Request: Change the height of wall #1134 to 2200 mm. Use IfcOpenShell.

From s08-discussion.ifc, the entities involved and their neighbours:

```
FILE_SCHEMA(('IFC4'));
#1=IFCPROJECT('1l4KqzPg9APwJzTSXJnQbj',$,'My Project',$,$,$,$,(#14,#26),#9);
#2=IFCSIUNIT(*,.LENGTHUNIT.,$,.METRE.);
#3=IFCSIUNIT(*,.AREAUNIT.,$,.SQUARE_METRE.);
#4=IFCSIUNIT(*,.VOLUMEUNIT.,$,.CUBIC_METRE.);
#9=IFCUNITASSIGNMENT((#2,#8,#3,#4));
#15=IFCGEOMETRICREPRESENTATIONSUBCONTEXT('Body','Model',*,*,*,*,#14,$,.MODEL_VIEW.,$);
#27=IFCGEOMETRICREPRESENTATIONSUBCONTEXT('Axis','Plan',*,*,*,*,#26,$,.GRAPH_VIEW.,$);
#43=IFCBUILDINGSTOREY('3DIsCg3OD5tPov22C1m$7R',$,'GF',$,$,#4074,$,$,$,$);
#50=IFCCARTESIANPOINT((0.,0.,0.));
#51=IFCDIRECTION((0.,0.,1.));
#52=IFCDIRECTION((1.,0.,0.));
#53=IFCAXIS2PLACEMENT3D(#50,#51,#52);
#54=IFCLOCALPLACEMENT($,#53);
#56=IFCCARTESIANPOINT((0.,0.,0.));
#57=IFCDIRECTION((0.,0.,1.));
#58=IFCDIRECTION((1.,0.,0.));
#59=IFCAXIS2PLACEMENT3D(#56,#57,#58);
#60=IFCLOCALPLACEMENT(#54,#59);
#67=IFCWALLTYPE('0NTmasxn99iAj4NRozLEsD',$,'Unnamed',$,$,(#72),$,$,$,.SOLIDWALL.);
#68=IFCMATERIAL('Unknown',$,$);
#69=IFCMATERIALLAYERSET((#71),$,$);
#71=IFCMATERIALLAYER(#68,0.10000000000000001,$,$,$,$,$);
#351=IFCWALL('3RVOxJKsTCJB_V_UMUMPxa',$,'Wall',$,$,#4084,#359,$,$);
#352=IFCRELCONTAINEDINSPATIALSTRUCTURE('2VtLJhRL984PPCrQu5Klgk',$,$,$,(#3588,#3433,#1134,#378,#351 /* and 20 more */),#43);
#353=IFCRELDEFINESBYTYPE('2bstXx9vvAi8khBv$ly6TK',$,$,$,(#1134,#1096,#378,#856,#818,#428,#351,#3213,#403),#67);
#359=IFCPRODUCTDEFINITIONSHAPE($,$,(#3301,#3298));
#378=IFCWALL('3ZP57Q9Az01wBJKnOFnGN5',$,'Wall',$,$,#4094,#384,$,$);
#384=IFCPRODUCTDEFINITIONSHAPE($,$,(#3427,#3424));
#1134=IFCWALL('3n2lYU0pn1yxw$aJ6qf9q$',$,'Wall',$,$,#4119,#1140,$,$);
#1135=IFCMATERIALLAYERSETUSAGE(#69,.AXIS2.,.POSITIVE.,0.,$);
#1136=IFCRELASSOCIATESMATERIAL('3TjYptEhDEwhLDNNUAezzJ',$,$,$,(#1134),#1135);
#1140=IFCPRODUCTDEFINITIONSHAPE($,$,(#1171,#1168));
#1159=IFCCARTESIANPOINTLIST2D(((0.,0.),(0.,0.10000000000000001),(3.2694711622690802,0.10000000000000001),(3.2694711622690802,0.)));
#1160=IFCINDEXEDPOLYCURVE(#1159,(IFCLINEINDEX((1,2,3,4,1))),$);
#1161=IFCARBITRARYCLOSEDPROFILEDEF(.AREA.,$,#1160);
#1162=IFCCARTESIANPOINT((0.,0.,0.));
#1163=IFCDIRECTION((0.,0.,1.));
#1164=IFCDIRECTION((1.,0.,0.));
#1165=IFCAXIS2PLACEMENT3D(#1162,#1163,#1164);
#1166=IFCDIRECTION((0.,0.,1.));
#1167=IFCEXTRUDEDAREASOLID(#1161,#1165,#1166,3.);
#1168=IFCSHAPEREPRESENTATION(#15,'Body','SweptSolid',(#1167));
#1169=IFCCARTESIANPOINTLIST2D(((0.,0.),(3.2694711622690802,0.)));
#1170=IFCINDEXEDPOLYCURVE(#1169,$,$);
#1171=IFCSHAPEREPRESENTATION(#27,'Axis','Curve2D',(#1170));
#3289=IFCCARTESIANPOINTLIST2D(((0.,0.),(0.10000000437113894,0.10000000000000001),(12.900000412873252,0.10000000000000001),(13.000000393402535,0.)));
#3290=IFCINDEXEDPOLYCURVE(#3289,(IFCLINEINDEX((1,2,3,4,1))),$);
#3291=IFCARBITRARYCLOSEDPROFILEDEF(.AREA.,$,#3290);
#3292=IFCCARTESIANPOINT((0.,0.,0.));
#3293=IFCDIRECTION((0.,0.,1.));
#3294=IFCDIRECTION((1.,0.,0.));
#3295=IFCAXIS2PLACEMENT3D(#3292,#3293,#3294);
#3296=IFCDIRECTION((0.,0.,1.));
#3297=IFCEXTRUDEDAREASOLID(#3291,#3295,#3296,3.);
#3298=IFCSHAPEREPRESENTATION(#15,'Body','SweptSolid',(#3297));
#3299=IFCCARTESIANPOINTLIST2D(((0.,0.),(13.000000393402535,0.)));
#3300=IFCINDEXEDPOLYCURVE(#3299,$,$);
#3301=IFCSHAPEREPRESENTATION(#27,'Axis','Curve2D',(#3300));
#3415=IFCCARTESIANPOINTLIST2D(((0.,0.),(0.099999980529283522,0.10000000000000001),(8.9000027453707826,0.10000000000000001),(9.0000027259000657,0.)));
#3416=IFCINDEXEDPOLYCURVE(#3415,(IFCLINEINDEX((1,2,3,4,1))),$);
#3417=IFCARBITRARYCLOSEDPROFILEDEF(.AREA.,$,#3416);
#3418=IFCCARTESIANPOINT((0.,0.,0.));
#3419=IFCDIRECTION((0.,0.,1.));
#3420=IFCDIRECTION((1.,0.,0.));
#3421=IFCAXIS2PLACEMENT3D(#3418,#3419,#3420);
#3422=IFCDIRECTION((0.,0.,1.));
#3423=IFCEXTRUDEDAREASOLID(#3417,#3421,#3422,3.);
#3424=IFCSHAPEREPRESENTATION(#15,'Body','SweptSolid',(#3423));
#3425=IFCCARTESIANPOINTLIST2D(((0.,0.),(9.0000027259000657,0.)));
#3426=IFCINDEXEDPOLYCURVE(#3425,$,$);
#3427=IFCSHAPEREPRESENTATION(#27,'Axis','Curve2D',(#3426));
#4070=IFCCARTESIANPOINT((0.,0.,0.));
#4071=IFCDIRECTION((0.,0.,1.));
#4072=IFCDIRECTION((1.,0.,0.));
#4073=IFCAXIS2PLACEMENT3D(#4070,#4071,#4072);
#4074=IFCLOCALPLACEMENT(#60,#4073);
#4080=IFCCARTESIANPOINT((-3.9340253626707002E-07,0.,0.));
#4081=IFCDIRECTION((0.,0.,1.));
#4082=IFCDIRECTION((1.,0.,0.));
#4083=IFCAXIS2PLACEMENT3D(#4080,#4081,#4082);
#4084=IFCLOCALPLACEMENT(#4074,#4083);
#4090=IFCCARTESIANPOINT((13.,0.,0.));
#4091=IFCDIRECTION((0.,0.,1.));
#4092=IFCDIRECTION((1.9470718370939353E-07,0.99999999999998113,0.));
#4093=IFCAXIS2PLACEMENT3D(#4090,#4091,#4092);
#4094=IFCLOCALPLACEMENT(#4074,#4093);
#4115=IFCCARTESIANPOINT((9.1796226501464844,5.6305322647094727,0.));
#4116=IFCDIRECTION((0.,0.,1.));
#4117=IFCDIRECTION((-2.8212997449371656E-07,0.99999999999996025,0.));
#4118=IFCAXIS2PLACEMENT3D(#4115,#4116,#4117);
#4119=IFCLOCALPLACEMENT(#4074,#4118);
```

```python
import ifcopenshell
import ifcopenshell.geom
import ifcopenshell.util.representation
import ifcopenshell.util.shape
import ifcopenshell.util.unit

model = ifcopenshell.open("s08-discussion.ifc")
unit_scale = ifcopenshell.util.unit.calculate_unit_scale(model)
settings = ifcopenshell.geom.settings()


def volume(element):
    """Net volume in cubic metres, openings subtracted."""
    shape = ifcopenshell.geom.create_shape(settings, element)
    return ifcopenshell.util.shape.get_volume(shape.geometry)


wall = model.by_guid("3n2lYU0pn1yxw$aJ6qf9q$")
before = volume(wall)

body = ifcopenshell.util.representation.get_representation(wall, "Model", "Body")
solid = body.Items[0]
old_height = solid.Depth
solid.Depth = 2.2 / unit_scale
after = volume(wall)

print(f"height {old_height:g} -> {solid.Depth:g}, volume {before:.3f} -> {after:.3f} m3")

model.write("s08-discussion_updated.ifc")
```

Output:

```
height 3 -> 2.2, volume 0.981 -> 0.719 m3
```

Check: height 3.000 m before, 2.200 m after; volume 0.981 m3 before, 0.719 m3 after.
